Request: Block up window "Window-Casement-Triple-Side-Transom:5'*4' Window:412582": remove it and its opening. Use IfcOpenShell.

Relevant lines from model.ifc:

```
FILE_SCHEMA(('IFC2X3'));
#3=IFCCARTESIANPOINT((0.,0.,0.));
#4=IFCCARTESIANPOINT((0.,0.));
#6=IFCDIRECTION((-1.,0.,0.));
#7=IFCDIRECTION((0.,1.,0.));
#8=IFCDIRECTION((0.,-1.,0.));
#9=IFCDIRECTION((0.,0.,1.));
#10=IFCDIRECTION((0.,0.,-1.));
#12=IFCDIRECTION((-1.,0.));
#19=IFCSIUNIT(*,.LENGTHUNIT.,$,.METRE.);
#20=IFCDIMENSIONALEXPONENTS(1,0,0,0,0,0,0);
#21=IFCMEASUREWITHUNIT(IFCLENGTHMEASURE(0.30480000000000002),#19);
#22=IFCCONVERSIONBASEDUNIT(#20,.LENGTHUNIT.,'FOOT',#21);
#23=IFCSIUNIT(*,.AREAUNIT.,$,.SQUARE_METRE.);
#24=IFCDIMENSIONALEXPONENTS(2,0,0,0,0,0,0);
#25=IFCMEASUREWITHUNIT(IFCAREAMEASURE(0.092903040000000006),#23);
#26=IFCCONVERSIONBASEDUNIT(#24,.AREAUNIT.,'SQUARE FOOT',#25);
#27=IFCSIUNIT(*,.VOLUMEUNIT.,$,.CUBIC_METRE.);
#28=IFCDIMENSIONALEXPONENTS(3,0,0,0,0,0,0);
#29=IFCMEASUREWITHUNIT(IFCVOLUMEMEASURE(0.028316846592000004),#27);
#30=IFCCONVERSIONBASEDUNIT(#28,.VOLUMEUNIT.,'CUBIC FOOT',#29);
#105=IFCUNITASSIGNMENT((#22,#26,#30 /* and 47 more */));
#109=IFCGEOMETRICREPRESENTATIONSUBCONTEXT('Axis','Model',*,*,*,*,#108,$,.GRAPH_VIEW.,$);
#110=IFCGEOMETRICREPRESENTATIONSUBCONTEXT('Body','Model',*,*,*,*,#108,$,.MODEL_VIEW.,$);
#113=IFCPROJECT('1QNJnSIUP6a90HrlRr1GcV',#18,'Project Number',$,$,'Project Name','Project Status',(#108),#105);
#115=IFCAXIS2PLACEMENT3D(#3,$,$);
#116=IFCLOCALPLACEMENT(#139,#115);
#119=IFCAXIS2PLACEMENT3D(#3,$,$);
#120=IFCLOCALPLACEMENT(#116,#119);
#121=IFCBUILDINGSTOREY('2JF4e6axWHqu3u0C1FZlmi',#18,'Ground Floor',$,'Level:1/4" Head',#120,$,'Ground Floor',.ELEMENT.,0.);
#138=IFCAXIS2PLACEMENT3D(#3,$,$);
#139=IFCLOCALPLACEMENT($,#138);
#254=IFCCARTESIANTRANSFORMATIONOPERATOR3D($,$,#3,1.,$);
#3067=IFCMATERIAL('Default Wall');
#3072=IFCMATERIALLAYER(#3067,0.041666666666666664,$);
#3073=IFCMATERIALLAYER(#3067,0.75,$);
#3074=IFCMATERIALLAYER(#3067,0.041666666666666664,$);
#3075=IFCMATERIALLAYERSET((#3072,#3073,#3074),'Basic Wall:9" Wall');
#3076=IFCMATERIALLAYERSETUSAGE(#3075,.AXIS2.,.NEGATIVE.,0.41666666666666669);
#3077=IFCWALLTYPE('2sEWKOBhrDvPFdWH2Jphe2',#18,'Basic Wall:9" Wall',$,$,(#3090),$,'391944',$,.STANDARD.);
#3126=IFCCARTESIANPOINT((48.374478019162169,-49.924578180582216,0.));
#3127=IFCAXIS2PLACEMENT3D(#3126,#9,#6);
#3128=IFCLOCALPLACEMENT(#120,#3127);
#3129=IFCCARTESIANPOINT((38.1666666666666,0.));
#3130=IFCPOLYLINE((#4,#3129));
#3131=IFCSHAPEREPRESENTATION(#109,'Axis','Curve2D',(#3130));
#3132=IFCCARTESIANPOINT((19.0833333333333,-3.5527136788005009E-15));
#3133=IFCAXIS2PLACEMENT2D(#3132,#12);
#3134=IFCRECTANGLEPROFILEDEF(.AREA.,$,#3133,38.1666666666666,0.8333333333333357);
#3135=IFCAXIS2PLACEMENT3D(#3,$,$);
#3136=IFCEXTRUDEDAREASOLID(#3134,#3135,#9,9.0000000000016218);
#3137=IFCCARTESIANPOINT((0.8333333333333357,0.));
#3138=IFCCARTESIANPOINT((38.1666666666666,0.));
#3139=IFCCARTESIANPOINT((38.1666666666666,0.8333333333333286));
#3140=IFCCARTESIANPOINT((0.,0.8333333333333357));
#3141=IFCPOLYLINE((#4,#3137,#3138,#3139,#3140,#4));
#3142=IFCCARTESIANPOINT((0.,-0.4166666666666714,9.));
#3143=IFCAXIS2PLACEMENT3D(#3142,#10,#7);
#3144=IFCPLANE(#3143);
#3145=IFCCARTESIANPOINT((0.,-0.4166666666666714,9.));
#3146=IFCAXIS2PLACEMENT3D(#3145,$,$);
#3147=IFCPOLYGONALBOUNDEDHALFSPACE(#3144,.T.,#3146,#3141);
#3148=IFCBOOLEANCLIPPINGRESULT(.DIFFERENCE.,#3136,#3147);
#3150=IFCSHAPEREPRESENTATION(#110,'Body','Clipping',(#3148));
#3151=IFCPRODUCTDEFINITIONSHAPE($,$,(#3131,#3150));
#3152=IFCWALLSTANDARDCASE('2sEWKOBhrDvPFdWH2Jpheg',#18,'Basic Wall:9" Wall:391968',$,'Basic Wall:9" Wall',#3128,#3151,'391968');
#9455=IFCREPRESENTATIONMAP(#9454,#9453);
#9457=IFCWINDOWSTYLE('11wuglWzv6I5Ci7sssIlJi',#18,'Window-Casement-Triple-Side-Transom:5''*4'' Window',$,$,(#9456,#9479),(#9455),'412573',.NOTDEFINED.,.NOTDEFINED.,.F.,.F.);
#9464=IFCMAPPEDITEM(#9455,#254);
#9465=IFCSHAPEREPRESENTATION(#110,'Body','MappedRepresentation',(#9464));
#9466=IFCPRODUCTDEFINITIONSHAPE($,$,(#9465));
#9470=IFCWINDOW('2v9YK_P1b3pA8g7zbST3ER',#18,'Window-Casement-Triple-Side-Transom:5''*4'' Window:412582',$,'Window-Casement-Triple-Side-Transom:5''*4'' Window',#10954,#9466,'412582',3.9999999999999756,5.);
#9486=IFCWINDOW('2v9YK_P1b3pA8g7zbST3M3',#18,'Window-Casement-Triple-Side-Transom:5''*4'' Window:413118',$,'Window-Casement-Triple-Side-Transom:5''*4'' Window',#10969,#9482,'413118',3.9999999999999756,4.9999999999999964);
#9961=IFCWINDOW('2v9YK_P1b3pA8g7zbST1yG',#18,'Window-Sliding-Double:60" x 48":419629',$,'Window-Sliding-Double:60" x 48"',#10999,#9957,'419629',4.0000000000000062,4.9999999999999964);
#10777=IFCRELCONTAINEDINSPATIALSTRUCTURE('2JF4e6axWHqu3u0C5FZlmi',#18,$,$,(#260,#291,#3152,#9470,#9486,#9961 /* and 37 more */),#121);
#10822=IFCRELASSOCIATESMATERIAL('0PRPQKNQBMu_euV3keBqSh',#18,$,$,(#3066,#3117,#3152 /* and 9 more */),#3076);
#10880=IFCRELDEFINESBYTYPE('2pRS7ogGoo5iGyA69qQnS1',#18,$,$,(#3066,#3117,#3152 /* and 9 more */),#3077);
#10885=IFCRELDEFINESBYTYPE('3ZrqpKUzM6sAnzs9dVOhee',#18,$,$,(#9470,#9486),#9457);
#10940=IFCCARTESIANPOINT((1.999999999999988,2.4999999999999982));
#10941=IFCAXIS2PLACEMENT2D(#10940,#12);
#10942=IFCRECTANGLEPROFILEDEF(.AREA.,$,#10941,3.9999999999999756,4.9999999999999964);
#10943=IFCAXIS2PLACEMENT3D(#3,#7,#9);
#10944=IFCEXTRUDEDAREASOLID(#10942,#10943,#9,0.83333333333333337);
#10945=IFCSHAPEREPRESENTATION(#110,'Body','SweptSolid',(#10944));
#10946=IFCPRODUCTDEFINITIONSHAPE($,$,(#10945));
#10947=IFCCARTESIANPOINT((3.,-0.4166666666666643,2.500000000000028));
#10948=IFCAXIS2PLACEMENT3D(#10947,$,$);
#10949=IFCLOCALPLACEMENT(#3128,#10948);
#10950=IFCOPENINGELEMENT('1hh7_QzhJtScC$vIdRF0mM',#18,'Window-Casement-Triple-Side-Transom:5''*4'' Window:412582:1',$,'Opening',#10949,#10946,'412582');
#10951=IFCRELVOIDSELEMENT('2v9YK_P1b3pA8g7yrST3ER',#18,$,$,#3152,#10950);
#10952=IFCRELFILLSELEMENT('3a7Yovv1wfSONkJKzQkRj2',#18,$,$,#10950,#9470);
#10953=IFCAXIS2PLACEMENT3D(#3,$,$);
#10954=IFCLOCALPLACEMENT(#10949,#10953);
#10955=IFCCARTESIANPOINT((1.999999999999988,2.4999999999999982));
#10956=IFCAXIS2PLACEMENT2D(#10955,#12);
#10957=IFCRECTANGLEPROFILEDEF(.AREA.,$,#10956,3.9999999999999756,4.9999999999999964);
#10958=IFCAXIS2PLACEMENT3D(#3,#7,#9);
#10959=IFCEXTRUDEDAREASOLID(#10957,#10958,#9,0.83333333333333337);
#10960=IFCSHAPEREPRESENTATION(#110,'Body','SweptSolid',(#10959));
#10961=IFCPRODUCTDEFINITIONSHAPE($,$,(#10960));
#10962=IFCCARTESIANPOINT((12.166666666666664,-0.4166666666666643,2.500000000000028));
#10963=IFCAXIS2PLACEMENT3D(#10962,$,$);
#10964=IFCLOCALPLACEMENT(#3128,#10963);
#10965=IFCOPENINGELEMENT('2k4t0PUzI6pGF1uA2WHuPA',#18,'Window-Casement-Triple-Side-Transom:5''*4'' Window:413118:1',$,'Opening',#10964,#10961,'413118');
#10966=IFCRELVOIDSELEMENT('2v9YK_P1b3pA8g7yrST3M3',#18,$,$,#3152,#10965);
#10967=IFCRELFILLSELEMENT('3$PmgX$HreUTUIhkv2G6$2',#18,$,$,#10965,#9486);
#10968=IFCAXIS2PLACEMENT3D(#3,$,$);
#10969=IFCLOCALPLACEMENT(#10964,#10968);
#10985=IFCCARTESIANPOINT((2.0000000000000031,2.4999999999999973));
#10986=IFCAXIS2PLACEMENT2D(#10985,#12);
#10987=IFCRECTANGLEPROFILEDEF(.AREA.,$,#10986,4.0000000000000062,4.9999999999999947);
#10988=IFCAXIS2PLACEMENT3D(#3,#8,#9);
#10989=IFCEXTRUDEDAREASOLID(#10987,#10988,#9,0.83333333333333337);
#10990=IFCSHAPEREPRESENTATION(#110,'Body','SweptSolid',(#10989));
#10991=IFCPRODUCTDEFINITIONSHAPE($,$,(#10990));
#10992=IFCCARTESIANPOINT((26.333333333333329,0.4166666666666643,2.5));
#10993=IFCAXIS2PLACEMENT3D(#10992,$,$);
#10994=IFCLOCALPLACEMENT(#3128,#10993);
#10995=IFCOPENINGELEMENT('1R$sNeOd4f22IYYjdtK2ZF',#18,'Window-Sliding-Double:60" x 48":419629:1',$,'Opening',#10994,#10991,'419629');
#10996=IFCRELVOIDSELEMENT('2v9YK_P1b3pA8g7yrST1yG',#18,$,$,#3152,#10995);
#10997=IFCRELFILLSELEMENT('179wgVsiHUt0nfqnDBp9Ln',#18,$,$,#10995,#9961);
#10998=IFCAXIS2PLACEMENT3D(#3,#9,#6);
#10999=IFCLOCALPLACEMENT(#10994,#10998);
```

```python
import ifcopenshell
import ifcopenshell.api.feature
import ifcopenshell.api.root
import ifcopenshell.geom
import ifcopenshell.util.shape

model = ifcopenshell.open("model.ifc")
settings = ifcopenshell.geom.settings()


def volume(element):
    """Net volume in cubic metres, openings subtracted."""
    shape = ifcopenshell.geom.create_shape(settings, element)
    return ifcopenshell.util.shape.get_volume(shape.geometry)


window = model.by_guid("2v9YK_P1b3pA8g7zbST3ER")
opening = window.FillsVoids[0].RelatingOpeningElement
wall = opening.VoidsElements[0].RelatingBuildingElement
before = volume(wall)

ifcopenshell.api.root.remove_product(model, product=window)
ifcopenshell.api.feature.remove_feature(model, feature=opening)

after = volume(wall)

print(f"wall volume {before:.3f} -> {after:.3f} m3")

model.write("model_edited.ifc")
```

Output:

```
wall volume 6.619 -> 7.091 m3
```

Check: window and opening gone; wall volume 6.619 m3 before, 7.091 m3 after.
